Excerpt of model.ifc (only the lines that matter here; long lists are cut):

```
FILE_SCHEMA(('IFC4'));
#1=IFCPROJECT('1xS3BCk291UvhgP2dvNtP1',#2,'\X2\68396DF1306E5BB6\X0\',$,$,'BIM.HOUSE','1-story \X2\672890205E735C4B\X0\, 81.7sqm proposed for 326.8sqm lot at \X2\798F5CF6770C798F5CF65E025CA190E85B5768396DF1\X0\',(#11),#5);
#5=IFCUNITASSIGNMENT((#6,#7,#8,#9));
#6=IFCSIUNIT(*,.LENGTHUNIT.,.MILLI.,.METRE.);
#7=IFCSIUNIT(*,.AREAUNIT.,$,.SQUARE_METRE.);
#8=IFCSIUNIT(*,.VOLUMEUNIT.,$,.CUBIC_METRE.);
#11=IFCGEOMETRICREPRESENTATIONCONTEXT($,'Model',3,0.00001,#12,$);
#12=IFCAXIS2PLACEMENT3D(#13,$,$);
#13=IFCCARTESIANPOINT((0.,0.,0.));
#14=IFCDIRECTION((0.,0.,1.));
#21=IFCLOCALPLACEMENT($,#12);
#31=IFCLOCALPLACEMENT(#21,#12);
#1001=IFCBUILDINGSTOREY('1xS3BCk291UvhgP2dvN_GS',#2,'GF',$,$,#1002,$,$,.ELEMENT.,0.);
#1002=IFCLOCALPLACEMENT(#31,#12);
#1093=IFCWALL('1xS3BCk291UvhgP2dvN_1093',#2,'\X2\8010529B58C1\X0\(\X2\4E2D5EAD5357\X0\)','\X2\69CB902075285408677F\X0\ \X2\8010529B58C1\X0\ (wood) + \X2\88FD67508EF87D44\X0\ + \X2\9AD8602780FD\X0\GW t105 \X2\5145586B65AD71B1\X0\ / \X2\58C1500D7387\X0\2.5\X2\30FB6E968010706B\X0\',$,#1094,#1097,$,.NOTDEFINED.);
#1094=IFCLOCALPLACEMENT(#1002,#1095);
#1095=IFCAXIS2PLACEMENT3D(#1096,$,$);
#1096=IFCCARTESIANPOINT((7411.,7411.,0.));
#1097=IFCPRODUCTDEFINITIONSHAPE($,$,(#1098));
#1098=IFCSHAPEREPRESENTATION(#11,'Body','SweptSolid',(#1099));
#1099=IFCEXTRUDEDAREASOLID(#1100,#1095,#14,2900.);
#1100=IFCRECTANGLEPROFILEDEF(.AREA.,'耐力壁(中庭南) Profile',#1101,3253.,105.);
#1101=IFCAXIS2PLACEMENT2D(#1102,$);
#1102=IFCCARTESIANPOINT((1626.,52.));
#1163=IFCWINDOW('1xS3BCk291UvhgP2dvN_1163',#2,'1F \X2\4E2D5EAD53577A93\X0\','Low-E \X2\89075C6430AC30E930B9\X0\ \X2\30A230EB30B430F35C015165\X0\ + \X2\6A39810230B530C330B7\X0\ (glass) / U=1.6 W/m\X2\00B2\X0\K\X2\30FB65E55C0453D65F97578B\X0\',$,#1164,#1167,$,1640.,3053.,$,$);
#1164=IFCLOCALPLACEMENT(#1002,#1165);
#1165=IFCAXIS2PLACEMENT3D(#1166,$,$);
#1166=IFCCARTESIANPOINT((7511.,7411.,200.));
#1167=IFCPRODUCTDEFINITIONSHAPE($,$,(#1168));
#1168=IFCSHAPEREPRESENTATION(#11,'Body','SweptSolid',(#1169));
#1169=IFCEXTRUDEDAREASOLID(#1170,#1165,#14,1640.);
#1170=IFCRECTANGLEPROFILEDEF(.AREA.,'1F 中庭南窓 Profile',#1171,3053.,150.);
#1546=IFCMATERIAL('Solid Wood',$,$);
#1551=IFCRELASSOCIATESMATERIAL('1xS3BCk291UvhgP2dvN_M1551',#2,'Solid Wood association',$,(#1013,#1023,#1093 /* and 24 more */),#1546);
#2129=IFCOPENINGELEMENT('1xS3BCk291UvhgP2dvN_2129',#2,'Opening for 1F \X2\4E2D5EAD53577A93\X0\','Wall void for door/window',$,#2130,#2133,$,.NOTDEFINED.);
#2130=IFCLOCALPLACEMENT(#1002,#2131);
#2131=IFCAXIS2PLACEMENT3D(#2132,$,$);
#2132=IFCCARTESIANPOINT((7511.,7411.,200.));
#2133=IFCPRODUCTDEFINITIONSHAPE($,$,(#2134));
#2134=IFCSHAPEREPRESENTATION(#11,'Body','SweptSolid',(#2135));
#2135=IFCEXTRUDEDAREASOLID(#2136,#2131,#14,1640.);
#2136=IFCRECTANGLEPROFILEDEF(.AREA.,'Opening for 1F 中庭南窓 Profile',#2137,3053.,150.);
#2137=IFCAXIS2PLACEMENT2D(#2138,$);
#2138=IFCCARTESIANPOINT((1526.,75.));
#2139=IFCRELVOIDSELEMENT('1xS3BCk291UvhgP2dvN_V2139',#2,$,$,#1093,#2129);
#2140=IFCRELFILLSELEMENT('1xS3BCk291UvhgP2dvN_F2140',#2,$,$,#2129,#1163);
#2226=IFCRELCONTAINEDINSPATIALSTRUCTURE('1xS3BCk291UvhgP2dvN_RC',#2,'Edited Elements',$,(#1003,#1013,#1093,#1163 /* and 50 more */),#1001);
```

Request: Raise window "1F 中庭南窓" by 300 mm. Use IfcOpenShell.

```python
import numpy as np
import ifcopenshell
import ifcopenshell.api.geometry
import ifcopenshell.util.placement
import ifcopenshell.util.unit

model = ifcopenshell.open("model.ifc")
unit_scale = ifcopenshell.util.unit.calculate_unit_scale(model)

window = model.by_guid("1xS3BCk291UvhgP2dvN_1163")
opening = window.FillsVoids[0].RelatingOpeningElement
dz = 300.0

shift = np.array([0.0, 0.0, dz])
# The window is not placed relative to its opening, so move both.
for product in (opening, window):
    matrix = ifcopenshell.util.placement.get_local_placement(product.ObjectPlacement)
    matrix[:3, 3] += shift
    ifcopenshell.api.geometry.edit_object_placement(model, product=product, matrix=matrix, is_si=False)

print(f"moved by {dz * unit_scale:+.3f} m")

model.write("model-out.ifc")
```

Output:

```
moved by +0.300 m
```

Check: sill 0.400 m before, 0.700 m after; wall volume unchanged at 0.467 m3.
